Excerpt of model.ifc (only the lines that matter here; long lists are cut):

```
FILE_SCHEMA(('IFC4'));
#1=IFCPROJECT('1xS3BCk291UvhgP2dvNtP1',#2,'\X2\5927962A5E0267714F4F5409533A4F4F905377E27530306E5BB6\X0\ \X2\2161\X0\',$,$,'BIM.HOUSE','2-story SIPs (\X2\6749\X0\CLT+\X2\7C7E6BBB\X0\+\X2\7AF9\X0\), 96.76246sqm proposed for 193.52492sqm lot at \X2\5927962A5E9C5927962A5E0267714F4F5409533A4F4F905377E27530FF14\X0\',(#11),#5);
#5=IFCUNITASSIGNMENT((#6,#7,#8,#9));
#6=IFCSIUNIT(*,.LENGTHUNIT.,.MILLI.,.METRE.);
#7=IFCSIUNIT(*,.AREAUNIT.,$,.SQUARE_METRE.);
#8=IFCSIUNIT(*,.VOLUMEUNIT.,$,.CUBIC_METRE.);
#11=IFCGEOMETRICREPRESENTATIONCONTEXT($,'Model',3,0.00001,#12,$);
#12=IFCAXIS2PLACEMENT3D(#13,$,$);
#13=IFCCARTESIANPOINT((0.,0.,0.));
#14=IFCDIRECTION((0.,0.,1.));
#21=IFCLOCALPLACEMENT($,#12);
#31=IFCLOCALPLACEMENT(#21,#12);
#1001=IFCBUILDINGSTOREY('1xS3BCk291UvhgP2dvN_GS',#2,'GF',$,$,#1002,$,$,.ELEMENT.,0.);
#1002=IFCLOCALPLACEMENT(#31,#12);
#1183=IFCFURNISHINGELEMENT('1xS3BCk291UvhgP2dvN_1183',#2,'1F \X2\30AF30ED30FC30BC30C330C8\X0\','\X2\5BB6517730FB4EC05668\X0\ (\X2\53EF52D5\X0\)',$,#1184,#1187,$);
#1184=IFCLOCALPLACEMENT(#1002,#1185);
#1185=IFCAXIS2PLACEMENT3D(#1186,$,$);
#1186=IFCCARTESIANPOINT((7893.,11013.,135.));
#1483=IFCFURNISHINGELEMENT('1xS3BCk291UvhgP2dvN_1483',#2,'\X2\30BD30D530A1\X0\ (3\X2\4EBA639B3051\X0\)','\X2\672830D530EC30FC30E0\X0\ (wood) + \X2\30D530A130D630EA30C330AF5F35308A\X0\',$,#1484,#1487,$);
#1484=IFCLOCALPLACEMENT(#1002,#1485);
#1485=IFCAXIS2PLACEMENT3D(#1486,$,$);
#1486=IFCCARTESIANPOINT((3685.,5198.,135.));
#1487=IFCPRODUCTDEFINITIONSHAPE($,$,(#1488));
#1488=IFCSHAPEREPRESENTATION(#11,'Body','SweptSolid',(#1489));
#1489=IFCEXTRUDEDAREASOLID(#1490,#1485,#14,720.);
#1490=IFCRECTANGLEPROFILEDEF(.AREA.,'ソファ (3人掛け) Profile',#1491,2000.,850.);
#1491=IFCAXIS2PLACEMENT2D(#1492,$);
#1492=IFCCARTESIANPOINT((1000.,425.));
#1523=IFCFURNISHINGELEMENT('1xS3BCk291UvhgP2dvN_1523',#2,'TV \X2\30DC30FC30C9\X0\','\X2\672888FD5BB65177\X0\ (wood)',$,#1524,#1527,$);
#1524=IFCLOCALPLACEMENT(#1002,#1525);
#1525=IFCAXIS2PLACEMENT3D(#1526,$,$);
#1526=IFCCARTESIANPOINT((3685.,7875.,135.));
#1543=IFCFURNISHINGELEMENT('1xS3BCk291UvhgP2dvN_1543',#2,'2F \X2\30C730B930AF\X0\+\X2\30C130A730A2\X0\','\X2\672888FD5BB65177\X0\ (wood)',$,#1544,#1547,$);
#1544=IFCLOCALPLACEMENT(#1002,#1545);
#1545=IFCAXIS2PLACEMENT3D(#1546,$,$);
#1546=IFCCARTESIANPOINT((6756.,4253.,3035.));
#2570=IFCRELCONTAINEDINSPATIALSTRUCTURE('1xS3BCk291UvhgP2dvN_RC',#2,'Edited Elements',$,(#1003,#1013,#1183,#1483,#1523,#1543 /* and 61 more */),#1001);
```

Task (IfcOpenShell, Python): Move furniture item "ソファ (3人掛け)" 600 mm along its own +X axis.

```python
import ifcopenshell
import ifcopenshell.api.geometry
import ifcopenshell.util.placement

model = ifcopenshell.open("model.ifc")

item = model.by_id(1483)
matrix = ifcopenshell.util.placement.get_local_placement(item.ObjectPlacement)
matrix[:3, 3] += matrix[:3, 0] * 600.0
ifcopenshell.api.geometry.edit_object_placement(model, product=item, matrix=matrix, is_si=False)

print(ifcopenshell.util.placement.get_local_placement(item.ObjectPlacement).round(3) + 0.0)

model.write("model_rev.ifc")
```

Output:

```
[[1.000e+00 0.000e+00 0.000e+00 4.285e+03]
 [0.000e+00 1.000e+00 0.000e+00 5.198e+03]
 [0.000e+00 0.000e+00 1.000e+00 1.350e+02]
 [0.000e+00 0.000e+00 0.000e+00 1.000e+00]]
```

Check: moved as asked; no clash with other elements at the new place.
